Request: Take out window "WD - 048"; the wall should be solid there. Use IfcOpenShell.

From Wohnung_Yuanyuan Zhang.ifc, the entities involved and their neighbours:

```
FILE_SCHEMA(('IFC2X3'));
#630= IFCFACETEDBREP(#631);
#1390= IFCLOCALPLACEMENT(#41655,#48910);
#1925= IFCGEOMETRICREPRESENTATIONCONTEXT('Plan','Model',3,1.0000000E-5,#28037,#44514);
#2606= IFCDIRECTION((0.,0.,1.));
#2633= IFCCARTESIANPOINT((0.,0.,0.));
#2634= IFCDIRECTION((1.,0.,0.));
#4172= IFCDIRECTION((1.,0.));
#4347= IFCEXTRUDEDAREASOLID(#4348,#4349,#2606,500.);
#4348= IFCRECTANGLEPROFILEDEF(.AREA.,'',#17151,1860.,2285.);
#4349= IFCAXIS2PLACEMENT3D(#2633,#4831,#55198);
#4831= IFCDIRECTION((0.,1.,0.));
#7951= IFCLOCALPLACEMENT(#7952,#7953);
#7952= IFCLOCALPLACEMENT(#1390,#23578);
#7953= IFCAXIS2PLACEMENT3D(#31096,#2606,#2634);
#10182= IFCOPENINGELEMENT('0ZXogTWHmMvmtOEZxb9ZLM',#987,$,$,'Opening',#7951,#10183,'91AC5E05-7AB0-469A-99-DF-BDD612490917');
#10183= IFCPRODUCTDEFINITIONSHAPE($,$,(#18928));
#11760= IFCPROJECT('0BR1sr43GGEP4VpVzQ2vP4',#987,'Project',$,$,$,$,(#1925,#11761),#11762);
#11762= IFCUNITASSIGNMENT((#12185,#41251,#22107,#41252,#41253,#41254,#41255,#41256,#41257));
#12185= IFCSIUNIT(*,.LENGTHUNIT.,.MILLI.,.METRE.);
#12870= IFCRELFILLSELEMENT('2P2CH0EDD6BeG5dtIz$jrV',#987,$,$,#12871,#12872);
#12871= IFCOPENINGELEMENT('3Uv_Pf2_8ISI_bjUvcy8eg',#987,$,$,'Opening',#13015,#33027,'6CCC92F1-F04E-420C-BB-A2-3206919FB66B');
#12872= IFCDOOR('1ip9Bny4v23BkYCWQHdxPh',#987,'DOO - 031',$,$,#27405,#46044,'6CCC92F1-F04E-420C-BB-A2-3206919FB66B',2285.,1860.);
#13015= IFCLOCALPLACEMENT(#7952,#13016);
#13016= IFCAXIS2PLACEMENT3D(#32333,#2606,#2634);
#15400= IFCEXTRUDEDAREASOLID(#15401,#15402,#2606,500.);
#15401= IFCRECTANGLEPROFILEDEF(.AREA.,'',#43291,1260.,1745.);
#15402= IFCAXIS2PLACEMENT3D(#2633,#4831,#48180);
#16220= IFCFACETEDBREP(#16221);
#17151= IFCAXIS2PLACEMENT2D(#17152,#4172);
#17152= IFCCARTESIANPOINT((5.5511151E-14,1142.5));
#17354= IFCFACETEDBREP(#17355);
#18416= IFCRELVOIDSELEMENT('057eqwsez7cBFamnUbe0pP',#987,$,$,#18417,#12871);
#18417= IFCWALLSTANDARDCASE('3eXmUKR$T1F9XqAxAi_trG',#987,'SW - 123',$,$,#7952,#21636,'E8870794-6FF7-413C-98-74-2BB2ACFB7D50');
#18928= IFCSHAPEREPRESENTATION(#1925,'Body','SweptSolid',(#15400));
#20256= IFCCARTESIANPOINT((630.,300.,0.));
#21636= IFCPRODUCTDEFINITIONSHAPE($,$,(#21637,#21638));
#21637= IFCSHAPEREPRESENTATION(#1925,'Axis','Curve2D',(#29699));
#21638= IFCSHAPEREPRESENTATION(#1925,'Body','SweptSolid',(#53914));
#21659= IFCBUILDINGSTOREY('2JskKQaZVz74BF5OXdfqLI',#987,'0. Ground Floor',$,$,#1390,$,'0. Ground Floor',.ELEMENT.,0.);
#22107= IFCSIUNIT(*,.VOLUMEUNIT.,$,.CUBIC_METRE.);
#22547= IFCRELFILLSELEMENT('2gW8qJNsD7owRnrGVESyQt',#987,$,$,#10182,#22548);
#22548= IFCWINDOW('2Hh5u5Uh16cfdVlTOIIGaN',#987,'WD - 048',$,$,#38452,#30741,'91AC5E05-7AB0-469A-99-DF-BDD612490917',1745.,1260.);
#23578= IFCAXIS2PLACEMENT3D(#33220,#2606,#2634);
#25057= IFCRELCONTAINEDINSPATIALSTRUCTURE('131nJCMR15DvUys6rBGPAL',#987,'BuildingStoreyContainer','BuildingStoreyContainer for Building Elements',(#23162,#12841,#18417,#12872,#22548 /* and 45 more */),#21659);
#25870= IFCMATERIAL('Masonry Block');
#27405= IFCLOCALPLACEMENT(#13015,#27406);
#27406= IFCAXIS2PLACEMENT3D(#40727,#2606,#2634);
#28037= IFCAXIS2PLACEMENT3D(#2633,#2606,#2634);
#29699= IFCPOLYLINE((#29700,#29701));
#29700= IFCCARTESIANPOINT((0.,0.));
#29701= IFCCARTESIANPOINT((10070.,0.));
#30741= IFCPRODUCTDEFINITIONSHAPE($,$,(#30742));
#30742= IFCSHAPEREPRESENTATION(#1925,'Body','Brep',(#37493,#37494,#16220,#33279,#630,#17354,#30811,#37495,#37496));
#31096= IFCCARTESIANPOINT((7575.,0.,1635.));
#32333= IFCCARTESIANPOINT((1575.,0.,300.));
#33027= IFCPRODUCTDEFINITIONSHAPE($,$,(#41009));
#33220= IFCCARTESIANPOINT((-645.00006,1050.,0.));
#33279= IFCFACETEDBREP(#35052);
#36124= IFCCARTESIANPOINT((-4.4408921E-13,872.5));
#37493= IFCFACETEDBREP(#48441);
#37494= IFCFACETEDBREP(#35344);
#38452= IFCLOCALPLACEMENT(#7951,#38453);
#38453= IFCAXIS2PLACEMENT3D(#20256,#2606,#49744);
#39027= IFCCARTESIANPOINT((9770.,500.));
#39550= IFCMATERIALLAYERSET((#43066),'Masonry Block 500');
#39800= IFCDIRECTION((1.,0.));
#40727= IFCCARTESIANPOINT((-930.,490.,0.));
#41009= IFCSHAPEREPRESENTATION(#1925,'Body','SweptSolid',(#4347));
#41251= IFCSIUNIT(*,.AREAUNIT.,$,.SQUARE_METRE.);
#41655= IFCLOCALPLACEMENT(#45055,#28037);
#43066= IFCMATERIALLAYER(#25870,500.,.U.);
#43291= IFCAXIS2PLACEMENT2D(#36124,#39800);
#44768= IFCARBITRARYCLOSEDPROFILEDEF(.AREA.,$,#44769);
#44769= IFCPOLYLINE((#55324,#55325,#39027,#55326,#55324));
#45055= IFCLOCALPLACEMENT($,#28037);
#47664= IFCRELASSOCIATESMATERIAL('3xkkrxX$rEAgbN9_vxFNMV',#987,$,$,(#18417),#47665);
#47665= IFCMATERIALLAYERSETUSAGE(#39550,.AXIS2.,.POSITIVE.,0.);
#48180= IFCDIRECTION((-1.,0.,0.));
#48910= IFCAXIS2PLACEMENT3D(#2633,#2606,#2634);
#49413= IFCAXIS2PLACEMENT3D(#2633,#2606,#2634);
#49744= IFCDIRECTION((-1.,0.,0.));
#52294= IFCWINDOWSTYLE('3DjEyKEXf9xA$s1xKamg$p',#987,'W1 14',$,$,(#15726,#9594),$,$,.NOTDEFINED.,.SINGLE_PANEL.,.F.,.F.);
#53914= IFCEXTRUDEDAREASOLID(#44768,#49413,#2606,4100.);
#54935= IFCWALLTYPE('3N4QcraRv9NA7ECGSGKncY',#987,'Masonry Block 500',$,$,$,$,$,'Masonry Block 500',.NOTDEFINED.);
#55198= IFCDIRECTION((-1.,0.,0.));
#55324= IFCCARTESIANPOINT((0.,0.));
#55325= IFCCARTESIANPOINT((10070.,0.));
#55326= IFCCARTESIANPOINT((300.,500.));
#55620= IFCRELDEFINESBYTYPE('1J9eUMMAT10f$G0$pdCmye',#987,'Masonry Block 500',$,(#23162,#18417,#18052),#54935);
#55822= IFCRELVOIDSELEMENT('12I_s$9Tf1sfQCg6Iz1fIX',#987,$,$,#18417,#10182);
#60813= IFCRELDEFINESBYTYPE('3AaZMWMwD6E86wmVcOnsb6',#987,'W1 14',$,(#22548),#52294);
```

```python
import ifcopenshell
import ifcopenshell.api.feature
import ifcopenshell.api.root
import ifcopenshell.geom
import ifcopenshell.util.shape

model = ifcopenshell.open("Wohnung_Yuanyuan Zhang.ifc")
settings = ifcopenshell.geom.settings()


def volume(element):
    """Net volume in cubic metres, openings subtracted."""
    shape = ifcopenshell.geom.create_shape(settings, element)
    return ifcopenshell.util.shape.get_volume(shape.geometry)


window = model.by_guid("2Hh5u5Uh16cfdVlTOIIGaN")
opening = window.FillsVoids[0].RelatingOpeningElement
wall = opening.VoidsElements[0].RelatingBuildingElement
before = volume(wall)

ifcopenshell.api.root.remove_product(model, product=window)
ifcopenshell.api.feature.remove_feature(model, feature=opening)

after = volume(wall)

print(f"wall volume {before:.3f} -> {after:.3f} m3")

model.write("Wohnung_Yuanyuan Zhang_v2.ifc")
```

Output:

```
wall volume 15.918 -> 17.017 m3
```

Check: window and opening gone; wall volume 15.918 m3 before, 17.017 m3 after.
